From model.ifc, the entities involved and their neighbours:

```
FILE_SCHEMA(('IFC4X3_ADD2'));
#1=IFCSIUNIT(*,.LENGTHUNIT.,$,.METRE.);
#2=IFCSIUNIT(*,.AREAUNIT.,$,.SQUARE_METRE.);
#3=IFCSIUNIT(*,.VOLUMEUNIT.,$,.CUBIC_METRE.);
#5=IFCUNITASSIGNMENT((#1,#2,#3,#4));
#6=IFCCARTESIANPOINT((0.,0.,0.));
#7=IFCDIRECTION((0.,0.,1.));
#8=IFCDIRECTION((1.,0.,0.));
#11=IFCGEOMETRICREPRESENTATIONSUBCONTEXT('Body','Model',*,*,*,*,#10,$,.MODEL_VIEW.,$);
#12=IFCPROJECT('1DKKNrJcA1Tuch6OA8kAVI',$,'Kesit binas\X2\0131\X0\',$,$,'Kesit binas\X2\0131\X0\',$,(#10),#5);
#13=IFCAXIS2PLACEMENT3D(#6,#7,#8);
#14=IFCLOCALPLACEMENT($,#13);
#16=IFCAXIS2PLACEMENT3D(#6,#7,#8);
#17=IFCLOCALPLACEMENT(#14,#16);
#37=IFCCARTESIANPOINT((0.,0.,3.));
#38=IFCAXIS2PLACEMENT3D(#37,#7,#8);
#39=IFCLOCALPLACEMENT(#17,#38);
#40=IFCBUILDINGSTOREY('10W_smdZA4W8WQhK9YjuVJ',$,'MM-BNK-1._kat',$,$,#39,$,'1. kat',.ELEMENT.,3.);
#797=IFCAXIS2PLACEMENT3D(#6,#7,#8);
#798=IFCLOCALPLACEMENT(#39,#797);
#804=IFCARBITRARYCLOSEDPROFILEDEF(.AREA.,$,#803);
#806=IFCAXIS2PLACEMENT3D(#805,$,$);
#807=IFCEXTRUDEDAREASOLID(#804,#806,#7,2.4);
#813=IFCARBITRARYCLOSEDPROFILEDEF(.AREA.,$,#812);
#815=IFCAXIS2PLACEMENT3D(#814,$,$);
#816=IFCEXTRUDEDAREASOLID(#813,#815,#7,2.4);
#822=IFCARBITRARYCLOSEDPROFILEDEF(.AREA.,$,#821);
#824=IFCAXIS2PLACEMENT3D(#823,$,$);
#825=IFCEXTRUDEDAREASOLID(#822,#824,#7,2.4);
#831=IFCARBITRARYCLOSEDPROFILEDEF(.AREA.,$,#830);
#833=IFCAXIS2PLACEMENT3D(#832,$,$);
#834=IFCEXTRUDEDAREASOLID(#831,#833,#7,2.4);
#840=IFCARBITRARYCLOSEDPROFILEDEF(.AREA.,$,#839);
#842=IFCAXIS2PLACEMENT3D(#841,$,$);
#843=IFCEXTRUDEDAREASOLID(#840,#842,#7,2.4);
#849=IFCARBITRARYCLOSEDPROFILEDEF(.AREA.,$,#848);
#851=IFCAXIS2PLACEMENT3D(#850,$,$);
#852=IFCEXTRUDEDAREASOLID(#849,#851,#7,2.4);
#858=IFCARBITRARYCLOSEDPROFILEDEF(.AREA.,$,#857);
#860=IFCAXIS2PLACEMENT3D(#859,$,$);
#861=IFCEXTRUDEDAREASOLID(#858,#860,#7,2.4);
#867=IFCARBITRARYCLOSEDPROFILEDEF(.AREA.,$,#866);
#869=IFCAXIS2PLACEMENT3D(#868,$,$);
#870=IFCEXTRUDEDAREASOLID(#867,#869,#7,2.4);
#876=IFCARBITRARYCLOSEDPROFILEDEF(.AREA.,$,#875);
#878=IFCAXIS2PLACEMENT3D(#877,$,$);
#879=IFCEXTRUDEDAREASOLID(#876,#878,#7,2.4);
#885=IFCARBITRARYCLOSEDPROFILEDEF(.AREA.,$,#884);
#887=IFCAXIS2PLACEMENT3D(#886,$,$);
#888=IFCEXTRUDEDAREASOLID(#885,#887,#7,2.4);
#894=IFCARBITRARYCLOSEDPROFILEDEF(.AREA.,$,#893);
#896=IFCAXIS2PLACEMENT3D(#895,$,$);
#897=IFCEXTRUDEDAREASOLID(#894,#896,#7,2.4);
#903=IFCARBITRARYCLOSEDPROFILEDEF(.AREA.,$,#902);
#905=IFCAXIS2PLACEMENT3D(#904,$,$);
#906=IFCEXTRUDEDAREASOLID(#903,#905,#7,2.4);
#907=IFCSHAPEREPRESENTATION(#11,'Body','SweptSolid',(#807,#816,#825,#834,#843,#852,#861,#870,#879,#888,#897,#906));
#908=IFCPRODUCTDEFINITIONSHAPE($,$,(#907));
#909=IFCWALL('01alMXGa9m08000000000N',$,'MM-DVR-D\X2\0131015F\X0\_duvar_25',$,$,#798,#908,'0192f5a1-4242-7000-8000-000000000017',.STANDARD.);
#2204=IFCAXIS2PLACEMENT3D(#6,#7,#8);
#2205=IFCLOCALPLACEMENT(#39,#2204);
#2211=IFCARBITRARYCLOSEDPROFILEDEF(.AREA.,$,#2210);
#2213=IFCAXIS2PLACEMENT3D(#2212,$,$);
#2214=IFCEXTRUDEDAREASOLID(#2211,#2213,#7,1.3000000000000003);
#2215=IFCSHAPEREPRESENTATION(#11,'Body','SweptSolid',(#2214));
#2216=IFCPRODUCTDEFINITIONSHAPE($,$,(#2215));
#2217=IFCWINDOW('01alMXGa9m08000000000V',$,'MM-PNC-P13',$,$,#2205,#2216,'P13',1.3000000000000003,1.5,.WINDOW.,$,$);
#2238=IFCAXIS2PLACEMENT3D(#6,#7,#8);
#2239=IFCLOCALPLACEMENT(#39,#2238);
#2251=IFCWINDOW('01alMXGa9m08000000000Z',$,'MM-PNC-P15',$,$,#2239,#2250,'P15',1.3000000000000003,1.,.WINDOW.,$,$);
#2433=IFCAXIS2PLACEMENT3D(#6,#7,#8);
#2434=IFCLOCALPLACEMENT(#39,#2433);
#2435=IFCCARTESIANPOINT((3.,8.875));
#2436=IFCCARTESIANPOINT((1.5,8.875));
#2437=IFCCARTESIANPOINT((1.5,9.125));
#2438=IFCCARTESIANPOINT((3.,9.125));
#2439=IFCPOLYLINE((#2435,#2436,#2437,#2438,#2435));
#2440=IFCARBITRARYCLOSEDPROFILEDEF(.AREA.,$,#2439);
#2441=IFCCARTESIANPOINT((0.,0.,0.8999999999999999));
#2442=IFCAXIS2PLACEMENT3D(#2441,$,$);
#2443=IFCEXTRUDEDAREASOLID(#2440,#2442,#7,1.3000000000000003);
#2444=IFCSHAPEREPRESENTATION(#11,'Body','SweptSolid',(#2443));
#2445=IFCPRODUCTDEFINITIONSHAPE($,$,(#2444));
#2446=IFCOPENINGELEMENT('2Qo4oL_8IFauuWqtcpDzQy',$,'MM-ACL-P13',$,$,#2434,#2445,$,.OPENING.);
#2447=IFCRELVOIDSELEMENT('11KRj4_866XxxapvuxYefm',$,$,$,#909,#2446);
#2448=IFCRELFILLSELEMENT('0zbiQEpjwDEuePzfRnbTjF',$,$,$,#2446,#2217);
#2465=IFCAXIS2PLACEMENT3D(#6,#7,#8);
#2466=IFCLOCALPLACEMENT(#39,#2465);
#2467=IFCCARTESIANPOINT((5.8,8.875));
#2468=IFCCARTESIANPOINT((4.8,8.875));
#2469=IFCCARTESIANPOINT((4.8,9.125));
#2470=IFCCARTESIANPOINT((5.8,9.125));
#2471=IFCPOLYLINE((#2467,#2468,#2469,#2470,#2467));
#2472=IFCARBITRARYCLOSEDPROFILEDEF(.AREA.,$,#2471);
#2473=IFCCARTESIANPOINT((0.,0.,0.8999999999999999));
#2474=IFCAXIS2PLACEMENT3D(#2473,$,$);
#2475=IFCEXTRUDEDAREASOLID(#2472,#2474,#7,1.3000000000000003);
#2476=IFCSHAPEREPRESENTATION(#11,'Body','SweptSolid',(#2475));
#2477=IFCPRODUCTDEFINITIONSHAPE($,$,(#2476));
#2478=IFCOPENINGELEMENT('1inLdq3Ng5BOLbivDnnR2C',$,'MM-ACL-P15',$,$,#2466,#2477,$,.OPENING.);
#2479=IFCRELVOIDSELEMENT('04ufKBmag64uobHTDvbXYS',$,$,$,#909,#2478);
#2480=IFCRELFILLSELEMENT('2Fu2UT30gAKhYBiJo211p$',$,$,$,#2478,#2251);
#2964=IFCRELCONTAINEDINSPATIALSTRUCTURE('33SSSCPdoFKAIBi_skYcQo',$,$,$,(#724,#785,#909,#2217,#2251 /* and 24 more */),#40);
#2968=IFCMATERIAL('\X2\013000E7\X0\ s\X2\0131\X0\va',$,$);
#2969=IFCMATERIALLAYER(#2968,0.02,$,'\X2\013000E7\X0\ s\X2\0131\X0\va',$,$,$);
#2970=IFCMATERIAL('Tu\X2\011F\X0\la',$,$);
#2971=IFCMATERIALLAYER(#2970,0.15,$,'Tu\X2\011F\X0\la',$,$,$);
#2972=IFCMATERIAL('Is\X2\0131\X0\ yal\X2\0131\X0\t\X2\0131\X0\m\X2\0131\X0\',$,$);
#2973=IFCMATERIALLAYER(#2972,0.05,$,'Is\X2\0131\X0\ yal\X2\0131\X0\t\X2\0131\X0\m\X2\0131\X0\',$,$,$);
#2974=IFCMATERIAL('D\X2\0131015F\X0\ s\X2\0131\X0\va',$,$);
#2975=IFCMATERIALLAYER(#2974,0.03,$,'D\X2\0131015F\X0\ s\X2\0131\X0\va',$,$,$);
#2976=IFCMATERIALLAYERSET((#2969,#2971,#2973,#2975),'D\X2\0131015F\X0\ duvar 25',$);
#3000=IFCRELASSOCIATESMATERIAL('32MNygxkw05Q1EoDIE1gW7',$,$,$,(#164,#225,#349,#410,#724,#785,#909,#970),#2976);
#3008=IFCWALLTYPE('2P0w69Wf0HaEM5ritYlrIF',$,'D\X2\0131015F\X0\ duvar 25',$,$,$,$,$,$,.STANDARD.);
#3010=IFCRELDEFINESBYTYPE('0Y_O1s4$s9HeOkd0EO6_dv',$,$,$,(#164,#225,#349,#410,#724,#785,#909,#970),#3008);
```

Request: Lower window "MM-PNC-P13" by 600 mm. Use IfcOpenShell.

```python
import numpy as np
import ifcopenshell
import ifcopenshell.api.geometry
import ifcopenshell.util.placement
import ifcopenshell.util.unit

model = ifcopenshell.open("model.ifc")
unit_scale = ifcopenshell.util.unit.calculate_unit_scale(model)

window = model.by_guid("01alMXGa9m08000000000V")
opening = window.FillsVoids[0].RelatingOpeningElement
dz = -0.6 / unit_scale

shift = np.array([0.0, 0.0, dz])
# The window is not placed relative to its opening, so move both.
for product in (opening, window):
    matrix = ifcopenshell.util.placement.get_local_placement(product.ObjectPlacement)
    matrix[:3, 3] += shift
    ifcopenshell.api.geometry.edit_object_placement(model, product=product, matrix=matrix, is_si=False)

print(f"moved by {dz * unit_scale:+.3f} m")

model.write("model-out.ifc")
```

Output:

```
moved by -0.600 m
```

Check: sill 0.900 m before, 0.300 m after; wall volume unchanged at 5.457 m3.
